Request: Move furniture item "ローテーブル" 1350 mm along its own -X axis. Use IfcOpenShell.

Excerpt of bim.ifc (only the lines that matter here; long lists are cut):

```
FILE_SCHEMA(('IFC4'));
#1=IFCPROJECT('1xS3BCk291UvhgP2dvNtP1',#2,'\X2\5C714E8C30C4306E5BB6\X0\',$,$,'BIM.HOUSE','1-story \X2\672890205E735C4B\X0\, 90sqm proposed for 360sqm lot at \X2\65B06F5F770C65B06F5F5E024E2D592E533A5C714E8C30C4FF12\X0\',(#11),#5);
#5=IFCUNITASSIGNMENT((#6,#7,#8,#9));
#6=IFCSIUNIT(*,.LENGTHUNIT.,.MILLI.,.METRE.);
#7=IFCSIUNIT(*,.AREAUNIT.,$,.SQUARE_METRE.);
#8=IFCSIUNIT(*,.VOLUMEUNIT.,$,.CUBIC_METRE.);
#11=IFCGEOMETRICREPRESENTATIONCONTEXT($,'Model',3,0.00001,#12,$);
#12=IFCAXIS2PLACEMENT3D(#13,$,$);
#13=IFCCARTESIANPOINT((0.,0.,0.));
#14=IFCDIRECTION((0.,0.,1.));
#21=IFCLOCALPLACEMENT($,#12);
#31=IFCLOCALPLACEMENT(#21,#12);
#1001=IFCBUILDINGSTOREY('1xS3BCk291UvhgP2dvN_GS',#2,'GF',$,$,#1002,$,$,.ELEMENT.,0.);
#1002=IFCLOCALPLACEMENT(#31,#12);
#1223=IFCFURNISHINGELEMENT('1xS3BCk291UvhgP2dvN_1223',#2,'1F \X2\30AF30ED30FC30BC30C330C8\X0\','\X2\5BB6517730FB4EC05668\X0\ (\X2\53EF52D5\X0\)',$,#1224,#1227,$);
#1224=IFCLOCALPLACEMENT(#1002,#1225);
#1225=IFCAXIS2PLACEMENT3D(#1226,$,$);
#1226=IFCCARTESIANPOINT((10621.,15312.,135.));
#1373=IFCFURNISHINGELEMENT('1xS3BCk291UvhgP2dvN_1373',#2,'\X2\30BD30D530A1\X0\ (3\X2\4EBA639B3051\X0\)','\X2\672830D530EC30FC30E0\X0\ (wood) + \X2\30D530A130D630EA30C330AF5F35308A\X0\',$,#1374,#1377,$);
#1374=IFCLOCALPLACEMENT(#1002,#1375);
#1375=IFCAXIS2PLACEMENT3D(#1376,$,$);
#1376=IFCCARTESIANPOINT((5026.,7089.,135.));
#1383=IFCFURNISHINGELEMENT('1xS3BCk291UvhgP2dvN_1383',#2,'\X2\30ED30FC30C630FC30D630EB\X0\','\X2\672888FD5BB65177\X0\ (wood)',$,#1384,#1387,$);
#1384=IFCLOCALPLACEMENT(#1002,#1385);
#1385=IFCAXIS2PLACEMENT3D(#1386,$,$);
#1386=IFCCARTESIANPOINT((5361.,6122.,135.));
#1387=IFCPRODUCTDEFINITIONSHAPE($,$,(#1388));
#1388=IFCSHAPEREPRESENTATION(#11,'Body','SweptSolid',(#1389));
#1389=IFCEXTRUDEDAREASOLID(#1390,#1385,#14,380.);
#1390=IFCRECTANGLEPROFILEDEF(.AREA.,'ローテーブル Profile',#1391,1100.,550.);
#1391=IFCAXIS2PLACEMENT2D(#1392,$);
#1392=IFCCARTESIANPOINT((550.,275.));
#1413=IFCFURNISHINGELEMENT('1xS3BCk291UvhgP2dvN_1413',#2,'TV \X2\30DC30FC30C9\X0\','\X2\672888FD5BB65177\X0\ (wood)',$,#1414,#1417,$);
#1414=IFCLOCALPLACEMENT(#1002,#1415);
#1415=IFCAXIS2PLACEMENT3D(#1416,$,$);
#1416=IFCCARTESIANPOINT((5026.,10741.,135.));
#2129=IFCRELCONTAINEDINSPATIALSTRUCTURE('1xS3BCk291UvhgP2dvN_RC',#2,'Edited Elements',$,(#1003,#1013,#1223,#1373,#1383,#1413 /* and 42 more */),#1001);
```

```python
import ifcopenshell
import ifcopenshell.api.geometry
import ifcopenshell.util.placement

model = ifcopenshell.open("bim.ifc")

item = model.by_guid("1xS3BCk291UvhgP2dvN_1383")
matrix = ifcopenshell.util.placement.get_local_placement(item.ObjectPlacement)
matrix[:3, 3] -= matrix[:3, 0] * 1350.0
ifcopenshell.api.geometry.edit_object_placement(model, product=item, matrix=matrix, is_si=False)

print(ifcopenshell.util.placement.get_local_placement(item.ObjectPlacement).round(3) + 0.0)

model.write("bim_rev.ifc")
```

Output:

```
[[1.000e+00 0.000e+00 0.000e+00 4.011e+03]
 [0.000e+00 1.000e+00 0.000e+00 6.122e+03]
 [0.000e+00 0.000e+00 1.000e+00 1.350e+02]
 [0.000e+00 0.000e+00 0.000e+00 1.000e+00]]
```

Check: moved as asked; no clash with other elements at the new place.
